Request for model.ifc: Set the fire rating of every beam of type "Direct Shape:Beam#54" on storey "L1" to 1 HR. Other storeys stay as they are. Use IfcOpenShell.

First a look at what the model holds.

```python
import ifcopenshell
import ifcopenshell.util.element

model = ifcopenshell.open("model.ifc")
print(model.schema)
storey = next(s for s in model.by_type("IfcBuildingStorey") if s.Name == "L1")
beams = [e for e in ifcopenshell.util.element.get_decomposition(storey) if e.is_a("IfcBeam")]
seen = {}
for e in beams:
    element_type = ifcopenshell.util.element.get_type(e)
    key = (element_type.Name if element_type != e and element_type else None, ifcopenshell.util.element.get_pset(e, "Pset_BeamCommon", "FireRating"))
    seen[key] = seen.get(key, 0) + 1
for (name, value), count in sorted(seen.items(), key=str):
    print(count, "x", name, "|", value)
```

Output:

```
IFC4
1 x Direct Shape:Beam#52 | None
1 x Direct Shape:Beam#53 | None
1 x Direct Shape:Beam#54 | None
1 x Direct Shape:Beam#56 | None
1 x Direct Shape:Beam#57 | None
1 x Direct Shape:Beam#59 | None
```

```python
import ifcopenshell
import ifcopenshell.api.pset
import ifcopenshell.util.element

model = ifcopenshell.open("model.ifc")

storey = next(s for s in model.by_type("IfcBuildingStorey") if s.Name == "L1")
beams = [e for e in ifcopenshell.util.element.get_decomposition(storey) if e.is_a("IfcBeam")]

count = 0
for e in beams:
    element_type = ifcopenshell.util.element.get_type(e)
    if element_type in (None, e) or element_type.Name != "Direct Shape:Beam#54":
        continue
    # add_pset returns the element's existing set when there is one.
    pset = ifcopenshell.api.pset.add_pset(model, product=e, name="Pset_BeamCommon")
    ifcopenshell.api.pset.edit_pset(model, pset=pset, properties={"FireRating": "1 HR"})
    count += 1

print(count, "beams updated")

model.write("model_rev.ifc")
```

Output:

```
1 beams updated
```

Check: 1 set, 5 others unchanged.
